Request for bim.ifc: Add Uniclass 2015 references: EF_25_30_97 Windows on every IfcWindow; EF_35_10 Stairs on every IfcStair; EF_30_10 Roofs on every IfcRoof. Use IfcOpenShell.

First a look at what the model holds.

```python
import ifcopenshell

model = ifcopenshell.open("bim.ifc")
print(model.schema)
print("classifications:", [c.Name for c in model.by_type("IfcClassification")])
for ifc_class in ("IfcDoor", "IfcRoof", "IfcStair", "IfcWall", "IfcWindow"):
    print(ifc_class, len(model.by_type(ifc_class)))
```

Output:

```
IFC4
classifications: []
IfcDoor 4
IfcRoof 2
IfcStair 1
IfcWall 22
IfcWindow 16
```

```python
import ifcopenshell
import ifcopenshell.api.classification

model = ifcopenshell.open("bim.ifc")

system = ifcopenshell.api.classification.add_classification(model, classification="Uniclass 2015")

codes = {
    "IfcWindow": ("EF_25_30_97", "Windows"),
    "IfcStair": ("EF_35_10", "Stairs"),
    "IfcRoof": ("EF_30_10", "Roofs"),
}
for ifc_class, (code, name) in codes.items():
    products = model.by_type(ifc_class)
    ifcopenshell.api.classification.add_reference(
        model, products=products, classification=system, identification=code, name=name
    )
    print(code, len(products))

model.write("bim_updated.ifc")
```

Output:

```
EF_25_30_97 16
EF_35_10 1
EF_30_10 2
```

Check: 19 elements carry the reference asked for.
